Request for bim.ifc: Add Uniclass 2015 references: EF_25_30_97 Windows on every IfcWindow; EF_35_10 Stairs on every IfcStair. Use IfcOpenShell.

First a look at what the model holds.

```python
import ifcopenshell

model = ifcopenshell.open("bim.ifc")
print(model.schema)
print("classifications:", [c.Name for c in model.by_type("IfcClassification")])
for ifc_class in ("IfcDoor", "IfcRoof", "IfcStair", "IfcWall", "IfcWindow"):
    print(ifc_class, len(model.by_type(ifc_class)))
```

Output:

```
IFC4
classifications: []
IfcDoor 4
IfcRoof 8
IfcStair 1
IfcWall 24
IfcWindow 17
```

```python
import ifcopenshell
import ifcopenshell.api.classification

model = ifcopenshell.open("bim.ifc")

system = ifcopenshell.api.classification.add_classification(model, classification="Uniclass 2015")

codes = {
    "IfcWindow": ("EF_25_30_97", "Windows"),
    "IfcStair": ("EF_35_10", "Stairs"),
}
for ifc_class, (code, name) in codes.items():
    products = model.by_type(ifc_class)
    ifcopenshell.api.classification.add_reference(
        model, products=products, classification=system, identification=code, name=name
    )
    print(code, len(products))

model.write("bim_edited.ifc")
```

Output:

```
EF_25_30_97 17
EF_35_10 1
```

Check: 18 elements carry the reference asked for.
